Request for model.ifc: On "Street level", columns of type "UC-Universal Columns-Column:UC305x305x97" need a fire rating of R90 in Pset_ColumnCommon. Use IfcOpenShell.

First a look at what the model holds.

```python
import ifcopenshell
import ifcopenshell.util.element

model = ifcopenshell.open("model.ifc")
print(model.schema)
storey = next(s for s in model.by_type("IfcBuildingStorey") if s.Name == "Street level")
columns = [e for e in ifcopenshell.util.element.get_decomposition(storey) if e.is_a("IfcColumn")]
seen = {}
for e in columns:
    element_type = ifcopenshell.util.element.get_type(e)
    key = (element_type.Name if element_type != e and element_type else None, ifcopenshell.util.element.get_pset(e, "Pset_ColumnCommon", "FireRating"))
    seen[key] = seen.get(key, 0) + 1
for (name, value), count in sorted(seen.items(), key=str):
    print(count, "x", name, "|", value)
```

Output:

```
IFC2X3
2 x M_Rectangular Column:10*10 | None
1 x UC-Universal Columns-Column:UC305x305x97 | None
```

```python
import ifcopenshell
import ifcopenshell.api.pset
import ifcopenshell.util.element

model = ifcopenshell.open("model.ifc")

storey = next(s for s in model.by_type("IfcBuildingStorey") if s.Name == "Street level")
columns = [e for e in ifcopenshell.util.element.get_decomposition(storey) if e.is_a("IfcColumn")]

count = 0
for e in columns:
    element_type = ifcopenshell.util.element.get_type(e)
    if element_type in (None, e) or element_type.Name != "UC-Universal Columns-Column:UC305x305x97":
        continue
    # add_pset returns the element's existing set when there is one.
    pset = ifcopenshell.api.pset.add_pset(model, product=e, name="Pset_ColumnCommon")
    ifcopenshell.api.pset.edit_pset(model, pset=pset, properties={"FireRating": "R90"})
    count += 1

print(count, "columns updated")

model.write("model_rev.ifc")
```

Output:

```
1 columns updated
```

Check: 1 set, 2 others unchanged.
